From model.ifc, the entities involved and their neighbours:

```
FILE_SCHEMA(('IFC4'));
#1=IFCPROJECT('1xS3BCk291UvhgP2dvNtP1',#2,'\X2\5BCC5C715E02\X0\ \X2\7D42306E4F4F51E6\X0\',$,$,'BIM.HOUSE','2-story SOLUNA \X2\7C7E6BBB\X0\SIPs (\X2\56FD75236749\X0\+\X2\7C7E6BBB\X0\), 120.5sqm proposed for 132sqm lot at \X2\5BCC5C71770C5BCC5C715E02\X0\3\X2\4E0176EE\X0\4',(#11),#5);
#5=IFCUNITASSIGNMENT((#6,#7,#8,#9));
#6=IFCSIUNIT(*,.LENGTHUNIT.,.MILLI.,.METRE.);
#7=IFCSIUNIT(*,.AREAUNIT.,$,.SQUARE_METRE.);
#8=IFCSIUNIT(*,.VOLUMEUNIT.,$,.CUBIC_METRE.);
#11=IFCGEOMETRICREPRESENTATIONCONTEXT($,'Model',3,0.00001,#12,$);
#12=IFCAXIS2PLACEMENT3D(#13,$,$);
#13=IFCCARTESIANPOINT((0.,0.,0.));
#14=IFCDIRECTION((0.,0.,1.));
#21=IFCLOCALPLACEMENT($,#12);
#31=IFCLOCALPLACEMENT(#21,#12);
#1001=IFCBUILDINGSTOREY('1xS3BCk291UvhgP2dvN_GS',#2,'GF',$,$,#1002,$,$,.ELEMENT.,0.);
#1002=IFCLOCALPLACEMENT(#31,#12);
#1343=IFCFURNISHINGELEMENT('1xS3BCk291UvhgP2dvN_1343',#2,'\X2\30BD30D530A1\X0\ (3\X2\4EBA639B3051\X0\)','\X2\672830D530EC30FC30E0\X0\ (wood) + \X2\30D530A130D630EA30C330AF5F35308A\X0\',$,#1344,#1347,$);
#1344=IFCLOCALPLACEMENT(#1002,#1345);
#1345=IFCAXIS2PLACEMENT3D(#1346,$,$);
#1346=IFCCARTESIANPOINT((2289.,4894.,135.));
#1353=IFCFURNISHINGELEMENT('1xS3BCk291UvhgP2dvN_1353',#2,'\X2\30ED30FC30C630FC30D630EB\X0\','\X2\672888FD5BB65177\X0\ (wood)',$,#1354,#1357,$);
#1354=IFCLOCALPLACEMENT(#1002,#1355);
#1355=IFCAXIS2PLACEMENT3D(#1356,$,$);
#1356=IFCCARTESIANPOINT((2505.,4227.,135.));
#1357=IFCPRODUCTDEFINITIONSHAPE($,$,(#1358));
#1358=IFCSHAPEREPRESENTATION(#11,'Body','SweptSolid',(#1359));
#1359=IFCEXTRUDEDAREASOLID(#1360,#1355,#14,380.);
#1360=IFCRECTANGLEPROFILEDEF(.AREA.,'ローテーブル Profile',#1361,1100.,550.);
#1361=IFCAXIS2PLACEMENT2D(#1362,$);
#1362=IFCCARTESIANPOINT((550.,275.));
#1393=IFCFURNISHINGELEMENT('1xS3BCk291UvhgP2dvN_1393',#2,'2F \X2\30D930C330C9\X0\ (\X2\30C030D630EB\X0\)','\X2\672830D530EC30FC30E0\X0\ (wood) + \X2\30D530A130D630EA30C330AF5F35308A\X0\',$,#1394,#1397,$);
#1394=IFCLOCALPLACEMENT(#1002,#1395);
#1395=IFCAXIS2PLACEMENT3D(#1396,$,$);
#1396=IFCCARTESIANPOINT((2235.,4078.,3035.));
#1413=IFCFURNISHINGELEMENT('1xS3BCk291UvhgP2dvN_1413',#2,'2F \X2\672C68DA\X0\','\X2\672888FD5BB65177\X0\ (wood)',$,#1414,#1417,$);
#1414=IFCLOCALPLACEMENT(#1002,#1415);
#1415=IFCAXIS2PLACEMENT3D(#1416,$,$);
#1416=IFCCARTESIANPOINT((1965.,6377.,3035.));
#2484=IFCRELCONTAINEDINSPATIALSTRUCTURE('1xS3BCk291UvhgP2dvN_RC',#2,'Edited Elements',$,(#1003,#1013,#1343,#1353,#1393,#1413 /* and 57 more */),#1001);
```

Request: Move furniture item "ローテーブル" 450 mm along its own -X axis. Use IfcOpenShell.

```python
import ifcopenshell
import ifcopenshell.api.geometry
import ifcopenshell.util.placement

model = ifcopenshell.open("model.ifc")

item = model.by_guid("1xS3BCk291UvhgP2dvN_1353")
matrix = ifcopenshell.util.placement.get_local_placement(item.ObjectPlacement)
matrix[:3, 3] -= matrix[:3, 0] * 450.0
ifcopenshell.api.geometry.edit_object_placement(model, product=item, matrix=matrix, is_si=False)

print(ifcopenshell.util.placement.get_local_placement(item.ObjectPlacement).round(3) + 0.0)

model.write("model_rev.ifc")
```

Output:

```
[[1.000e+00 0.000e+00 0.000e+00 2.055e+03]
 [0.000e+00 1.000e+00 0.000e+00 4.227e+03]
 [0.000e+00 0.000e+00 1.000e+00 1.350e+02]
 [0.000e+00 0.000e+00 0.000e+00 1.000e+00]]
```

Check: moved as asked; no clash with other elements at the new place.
